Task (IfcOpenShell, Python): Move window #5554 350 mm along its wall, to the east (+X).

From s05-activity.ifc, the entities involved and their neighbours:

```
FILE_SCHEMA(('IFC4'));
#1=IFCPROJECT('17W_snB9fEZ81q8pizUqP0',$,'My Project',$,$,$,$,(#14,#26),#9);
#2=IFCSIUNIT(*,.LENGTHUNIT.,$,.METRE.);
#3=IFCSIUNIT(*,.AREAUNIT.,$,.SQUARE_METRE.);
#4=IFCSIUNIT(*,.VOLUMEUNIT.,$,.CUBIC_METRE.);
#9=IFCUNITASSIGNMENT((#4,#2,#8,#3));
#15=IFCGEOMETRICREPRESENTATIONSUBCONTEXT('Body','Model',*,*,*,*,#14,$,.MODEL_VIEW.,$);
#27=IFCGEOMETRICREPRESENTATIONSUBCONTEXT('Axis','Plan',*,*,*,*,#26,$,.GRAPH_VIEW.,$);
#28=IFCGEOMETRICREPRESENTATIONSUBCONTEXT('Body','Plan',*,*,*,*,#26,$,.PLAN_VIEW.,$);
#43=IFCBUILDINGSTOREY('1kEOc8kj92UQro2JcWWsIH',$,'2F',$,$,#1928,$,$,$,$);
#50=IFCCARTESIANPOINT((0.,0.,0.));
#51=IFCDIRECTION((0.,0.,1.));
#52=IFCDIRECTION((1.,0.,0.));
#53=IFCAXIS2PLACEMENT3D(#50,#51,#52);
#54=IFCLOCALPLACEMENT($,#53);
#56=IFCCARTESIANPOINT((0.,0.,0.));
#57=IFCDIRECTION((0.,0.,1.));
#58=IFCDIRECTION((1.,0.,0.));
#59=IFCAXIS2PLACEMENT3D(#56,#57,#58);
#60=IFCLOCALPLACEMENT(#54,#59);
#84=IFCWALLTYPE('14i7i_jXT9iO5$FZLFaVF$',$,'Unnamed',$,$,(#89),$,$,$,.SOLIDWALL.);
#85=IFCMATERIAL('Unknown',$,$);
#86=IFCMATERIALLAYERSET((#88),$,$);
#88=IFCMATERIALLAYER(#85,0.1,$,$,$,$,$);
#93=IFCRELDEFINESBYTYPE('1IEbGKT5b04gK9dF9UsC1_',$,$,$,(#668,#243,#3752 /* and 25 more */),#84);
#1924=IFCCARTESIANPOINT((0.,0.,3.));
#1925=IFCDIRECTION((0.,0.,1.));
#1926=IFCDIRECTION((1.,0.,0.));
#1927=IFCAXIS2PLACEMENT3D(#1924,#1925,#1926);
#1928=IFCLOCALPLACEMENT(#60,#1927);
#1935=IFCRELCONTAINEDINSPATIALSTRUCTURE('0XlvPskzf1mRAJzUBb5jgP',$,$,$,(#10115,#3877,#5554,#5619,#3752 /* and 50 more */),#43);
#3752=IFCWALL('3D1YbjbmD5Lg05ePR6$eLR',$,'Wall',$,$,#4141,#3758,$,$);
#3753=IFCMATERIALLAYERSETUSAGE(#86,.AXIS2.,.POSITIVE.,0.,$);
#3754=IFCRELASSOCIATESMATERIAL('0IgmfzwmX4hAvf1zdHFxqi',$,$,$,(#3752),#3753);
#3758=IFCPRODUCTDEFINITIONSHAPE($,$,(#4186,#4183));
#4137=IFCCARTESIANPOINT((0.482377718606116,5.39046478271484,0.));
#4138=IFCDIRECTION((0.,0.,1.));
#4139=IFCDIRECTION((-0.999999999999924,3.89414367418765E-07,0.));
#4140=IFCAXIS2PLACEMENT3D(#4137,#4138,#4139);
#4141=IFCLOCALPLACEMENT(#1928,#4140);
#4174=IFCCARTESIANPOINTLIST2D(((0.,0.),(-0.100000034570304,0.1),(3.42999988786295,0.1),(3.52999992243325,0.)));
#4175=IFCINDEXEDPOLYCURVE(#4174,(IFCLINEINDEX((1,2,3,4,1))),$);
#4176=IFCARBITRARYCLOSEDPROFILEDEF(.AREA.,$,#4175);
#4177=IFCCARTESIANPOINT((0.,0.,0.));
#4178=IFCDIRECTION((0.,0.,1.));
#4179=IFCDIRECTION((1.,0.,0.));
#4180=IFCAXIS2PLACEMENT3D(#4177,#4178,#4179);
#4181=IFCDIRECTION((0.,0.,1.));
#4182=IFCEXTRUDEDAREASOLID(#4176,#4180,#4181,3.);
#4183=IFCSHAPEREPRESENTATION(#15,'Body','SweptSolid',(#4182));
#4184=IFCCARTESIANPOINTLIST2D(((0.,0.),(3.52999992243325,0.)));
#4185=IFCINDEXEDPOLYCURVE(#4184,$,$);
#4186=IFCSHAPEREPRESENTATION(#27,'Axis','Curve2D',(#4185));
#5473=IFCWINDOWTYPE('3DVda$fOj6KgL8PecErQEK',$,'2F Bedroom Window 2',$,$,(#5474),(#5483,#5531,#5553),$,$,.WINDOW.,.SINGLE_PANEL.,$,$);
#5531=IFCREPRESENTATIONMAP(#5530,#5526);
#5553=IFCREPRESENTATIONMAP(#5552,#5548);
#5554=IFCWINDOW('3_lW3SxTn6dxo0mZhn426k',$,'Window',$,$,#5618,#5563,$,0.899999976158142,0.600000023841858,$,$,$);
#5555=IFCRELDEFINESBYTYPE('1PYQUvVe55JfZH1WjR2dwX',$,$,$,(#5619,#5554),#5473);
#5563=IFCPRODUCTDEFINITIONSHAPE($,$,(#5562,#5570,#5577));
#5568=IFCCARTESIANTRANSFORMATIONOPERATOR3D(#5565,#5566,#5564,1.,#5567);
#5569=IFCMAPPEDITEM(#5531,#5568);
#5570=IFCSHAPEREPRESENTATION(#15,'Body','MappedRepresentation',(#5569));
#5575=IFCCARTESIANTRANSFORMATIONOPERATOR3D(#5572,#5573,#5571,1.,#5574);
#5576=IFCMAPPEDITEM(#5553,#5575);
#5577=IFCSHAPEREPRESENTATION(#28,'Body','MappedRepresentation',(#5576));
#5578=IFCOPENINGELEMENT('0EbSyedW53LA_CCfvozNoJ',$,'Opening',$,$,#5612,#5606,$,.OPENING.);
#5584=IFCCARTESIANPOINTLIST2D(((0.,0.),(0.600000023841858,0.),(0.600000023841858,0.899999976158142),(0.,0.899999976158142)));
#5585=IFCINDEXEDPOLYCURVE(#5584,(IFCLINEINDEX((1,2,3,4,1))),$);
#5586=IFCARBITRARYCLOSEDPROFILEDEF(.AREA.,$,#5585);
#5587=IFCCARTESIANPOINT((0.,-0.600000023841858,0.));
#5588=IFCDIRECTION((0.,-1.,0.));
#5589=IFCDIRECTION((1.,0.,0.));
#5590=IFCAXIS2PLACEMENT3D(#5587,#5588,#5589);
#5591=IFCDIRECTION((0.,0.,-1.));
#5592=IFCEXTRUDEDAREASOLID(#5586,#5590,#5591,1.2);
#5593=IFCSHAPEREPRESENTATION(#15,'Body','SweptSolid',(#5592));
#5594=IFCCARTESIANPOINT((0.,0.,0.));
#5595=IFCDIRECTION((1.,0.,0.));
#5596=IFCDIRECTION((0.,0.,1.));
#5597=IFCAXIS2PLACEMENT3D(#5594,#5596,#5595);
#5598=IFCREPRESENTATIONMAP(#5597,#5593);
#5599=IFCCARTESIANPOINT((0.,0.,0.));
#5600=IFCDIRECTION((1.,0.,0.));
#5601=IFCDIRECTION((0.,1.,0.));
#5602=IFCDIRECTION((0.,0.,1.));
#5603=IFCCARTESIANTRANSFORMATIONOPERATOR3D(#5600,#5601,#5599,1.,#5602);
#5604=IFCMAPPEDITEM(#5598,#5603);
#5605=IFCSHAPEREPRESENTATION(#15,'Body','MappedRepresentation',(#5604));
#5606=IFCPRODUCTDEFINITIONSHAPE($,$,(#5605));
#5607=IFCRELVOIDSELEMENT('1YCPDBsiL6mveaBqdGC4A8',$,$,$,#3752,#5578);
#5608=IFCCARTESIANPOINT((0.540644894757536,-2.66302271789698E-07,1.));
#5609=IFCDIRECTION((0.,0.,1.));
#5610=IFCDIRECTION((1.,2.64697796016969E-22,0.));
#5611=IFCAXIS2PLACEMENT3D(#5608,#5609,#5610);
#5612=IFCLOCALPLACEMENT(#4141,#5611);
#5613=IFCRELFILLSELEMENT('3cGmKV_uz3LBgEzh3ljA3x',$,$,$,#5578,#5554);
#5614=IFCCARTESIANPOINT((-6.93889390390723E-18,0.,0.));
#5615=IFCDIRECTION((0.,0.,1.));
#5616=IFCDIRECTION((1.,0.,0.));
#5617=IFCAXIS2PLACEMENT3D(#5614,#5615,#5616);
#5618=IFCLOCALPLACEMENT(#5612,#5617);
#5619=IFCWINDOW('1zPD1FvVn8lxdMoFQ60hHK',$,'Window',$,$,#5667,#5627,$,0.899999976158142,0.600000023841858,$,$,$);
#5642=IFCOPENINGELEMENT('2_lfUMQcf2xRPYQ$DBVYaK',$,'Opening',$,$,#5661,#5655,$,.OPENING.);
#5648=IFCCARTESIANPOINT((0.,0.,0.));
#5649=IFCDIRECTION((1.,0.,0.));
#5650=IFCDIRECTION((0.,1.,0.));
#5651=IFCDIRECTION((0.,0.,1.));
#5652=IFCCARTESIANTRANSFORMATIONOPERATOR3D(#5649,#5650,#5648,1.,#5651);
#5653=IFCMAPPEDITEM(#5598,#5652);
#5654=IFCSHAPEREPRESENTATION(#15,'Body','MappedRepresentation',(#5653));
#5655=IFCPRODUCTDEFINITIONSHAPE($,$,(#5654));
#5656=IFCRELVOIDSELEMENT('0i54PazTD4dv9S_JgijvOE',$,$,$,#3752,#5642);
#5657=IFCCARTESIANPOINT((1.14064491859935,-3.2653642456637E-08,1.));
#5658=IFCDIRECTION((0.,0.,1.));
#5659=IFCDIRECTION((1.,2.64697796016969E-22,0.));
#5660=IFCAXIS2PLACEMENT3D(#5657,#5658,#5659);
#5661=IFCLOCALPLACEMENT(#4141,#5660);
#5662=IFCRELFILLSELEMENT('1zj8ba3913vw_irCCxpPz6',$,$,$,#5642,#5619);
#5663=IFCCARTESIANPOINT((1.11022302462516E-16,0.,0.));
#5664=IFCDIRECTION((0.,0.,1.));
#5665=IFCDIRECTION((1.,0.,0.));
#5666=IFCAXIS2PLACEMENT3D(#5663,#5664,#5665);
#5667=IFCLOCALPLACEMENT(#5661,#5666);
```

```python
import ifcopenshell
import ifcopenshell.api.geometry
import ifcopenshell.util.placement
import ifcopenshell.util.unit

model = ifcopenshell.open("s05-activity.ifc")
unit_scale = ifcopenshell.util.unit.calculate_unit_scale(model)

window = model.by_id(5554)
opening = window.FillsVoids[0].RelatingOpeningElement
wall = opening.VoidsElements[0].RelatingBuildingElement

wall_matrix = ifcopenshell.util.placement.get_local_placement(wall.ObjectPlacement)
shift = wall_matrix[:3, 0] * -0.35 / unit_scale
before = ifcopenshell.util.placement.get_local_placement(window.ObjectPlacement)[:3, 3].copy()

# The window is placed relative to its opening, so it follows when the opening moves.
matrix = ifcopenshell.util.placement.get_local_placement(opening.ObjectPlacement)
matrix[:3, 3] += shift
ifcopenshell.api.geometry.edit_object_placement(
    model, product=opening, matrix=matrix, is_si=False, should_transform_children=True
)

after = ifcopenshell.util.placement.get_local_placement(window.ObjectPlacement)[:3, 3]
print("window moved by", (after - before).round(3) + 0.0)

model.write("s05-activity_rev.ifc")
```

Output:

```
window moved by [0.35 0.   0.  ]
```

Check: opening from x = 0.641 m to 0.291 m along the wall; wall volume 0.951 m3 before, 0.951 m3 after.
